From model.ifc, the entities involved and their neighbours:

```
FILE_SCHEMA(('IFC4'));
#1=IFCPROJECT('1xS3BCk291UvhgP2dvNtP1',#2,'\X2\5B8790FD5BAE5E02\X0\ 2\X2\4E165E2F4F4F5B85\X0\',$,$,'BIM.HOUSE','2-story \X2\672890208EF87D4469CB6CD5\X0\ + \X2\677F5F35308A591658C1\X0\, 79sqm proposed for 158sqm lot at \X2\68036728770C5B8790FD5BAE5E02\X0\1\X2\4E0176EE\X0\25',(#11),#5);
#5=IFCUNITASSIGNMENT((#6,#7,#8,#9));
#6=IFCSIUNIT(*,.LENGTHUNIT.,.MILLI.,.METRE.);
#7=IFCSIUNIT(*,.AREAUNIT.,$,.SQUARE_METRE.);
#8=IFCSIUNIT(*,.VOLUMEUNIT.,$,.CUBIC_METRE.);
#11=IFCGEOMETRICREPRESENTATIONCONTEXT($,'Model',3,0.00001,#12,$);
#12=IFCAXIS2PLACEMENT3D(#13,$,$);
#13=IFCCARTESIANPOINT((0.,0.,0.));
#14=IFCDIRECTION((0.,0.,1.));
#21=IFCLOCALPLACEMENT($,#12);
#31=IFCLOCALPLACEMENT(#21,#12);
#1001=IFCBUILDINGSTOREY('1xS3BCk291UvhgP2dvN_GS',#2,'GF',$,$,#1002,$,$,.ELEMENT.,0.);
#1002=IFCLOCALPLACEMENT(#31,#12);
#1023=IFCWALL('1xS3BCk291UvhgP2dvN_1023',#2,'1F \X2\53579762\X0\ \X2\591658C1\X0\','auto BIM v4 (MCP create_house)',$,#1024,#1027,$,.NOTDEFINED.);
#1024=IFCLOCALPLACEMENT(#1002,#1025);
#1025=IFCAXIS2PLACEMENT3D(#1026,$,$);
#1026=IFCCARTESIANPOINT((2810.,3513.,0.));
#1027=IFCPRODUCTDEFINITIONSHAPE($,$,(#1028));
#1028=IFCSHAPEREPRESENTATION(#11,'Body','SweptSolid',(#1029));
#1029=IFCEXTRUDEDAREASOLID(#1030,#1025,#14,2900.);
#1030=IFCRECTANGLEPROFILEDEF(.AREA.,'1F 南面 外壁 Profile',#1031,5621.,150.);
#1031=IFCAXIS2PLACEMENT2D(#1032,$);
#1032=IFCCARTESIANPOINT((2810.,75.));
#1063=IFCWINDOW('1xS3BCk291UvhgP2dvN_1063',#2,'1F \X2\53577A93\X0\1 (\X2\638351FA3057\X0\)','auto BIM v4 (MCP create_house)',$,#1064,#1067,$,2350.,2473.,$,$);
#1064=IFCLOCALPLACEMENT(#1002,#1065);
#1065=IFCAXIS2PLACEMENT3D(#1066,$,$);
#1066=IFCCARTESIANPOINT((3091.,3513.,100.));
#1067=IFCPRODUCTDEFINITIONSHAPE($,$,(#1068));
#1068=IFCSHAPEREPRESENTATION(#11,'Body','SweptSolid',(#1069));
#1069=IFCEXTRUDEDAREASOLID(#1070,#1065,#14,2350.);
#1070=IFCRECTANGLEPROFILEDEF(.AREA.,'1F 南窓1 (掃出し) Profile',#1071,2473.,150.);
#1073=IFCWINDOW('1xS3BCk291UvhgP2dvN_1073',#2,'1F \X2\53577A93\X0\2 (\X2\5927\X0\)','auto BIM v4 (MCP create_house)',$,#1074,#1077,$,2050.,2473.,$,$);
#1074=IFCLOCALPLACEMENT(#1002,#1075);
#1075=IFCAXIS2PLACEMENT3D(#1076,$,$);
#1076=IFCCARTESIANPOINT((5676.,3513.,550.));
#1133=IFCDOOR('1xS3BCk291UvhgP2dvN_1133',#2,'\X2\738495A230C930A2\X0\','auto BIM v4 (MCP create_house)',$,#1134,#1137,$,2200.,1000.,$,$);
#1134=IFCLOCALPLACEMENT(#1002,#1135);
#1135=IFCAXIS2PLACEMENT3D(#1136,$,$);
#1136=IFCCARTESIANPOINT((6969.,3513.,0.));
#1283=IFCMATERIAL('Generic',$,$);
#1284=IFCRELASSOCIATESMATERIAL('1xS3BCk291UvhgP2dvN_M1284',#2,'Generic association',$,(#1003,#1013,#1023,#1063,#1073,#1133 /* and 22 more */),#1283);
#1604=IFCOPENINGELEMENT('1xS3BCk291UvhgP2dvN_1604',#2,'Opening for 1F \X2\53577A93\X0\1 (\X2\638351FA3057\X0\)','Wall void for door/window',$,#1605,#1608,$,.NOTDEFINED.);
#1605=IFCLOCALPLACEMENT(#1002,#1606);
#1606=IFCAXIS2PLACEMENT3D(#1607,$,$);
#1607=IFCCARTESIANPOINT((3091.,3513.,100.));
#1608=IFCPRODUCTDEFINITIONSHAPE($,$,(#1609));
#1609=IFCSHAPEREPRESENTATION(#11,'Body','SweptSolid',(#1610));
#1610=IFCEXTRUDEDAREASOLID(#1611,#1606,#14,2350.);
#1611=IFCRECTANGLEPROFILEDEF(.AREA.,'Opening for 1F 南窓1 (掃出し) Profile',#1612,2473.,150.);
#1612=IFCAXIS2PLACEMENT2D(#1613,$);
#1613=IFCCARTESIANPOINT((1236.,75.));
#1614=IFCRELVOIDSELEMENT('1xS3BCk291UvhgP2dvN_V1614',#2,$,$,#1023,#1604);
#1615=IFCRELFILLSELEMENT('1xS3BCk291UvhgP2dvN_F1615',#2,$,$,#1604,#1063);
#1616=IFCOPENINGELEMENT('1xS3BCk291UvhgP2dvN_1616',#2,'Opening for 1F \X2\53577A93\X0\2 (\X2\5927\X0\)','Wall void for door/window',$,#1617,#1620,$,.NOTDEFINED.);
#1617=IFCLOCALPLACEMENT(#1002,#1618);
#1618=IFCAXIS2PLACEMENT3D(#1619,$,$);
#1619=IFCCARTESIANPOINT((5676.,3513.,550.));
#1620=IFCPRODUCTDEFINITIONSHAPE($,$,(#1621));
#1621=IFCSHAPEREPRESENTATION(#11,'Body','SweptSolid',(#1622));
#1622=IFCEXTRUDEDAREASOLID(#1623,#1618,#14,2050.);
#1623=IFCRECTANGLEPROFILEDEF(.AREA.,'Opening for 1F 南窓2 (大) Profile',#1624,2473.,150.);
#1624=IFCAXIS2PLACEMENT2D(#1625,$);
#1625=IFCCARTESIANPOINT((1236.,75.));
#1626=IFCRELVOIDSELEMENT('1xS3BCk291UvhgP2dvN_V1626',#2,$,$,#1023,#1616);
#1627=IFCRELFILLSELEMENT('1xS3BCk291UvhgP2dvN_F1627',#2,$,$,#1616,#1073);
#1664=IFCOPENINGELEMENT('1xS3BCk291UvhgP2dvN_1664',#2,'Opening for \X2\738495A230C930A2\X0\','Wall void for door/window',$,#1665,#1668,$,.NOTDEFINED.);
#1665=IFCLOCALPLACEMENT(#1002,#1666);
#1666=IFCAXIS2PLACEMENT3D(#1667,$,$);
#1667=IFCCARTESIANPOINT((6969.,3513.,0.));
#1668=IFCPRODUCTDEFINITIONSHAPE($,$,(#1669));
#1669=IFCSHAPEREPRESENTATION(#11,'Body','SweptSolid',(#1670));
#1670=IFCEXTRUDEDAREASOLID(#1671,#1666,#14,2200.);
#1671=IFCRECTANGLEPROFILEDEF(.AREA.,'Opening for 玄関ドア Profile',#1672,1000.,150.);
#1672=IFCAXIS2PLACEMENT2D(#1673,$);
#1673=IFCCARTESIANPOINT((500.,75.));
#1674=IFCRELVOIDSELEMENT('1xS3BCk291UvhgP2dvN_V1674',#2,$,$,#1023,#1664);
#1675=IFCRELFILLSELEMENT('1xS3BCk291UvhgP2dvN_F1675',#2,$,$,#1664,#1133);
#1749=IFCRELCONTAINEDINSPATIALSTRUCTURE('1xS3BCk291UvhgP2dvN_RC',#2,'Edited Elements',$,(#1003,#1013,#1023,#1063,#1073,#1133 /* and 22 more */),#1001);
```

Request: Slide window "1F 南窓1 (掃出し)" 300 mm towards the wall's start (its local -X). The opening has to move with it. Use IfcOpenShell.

```python
import ifcopenshell
import ifcopenshell.api.geometry
import ifcopenshell.util.placement

model = ifcopenshell.open("model.ifc")

window = model.by_id(1063)
opening = window.FillsVoids[0].RelatingOpeningElement
wall = opening.VoidsElements[0].RelatingBuildingElement

wall_matrix = ifcopenshell.util.placement.get_local_placement(wall.ObjectPlacement)
shift = wall_matrix[:3, 0] * -300.0
before = ifcopenshell.util.placement.get_local_placement(window.ObjectPlacement)[:3, 3].copy()

# The window is not placed relative to its opening, so move both.
for product in (opening, window):
    matrix = ifcopenshell.util.placement.get_local_placement(product.ObjectPlacement)
    matrix[:3, 3] += shift
    ifcopenshell.api.geometry.edit_object_placement(model, product=product, matrix=matrix, is_si=False)

after = ifcopenshell.util.placement.get_local_placement(window.ObjectPlacement)[:3, 3]
print("window moved by", (after - before).round(3) + 0.0)

model.write("model_rev.ifc")
```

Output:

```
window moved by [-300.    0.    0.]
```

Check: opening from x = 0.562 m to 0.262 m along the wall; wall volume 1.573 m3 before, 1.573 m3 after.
